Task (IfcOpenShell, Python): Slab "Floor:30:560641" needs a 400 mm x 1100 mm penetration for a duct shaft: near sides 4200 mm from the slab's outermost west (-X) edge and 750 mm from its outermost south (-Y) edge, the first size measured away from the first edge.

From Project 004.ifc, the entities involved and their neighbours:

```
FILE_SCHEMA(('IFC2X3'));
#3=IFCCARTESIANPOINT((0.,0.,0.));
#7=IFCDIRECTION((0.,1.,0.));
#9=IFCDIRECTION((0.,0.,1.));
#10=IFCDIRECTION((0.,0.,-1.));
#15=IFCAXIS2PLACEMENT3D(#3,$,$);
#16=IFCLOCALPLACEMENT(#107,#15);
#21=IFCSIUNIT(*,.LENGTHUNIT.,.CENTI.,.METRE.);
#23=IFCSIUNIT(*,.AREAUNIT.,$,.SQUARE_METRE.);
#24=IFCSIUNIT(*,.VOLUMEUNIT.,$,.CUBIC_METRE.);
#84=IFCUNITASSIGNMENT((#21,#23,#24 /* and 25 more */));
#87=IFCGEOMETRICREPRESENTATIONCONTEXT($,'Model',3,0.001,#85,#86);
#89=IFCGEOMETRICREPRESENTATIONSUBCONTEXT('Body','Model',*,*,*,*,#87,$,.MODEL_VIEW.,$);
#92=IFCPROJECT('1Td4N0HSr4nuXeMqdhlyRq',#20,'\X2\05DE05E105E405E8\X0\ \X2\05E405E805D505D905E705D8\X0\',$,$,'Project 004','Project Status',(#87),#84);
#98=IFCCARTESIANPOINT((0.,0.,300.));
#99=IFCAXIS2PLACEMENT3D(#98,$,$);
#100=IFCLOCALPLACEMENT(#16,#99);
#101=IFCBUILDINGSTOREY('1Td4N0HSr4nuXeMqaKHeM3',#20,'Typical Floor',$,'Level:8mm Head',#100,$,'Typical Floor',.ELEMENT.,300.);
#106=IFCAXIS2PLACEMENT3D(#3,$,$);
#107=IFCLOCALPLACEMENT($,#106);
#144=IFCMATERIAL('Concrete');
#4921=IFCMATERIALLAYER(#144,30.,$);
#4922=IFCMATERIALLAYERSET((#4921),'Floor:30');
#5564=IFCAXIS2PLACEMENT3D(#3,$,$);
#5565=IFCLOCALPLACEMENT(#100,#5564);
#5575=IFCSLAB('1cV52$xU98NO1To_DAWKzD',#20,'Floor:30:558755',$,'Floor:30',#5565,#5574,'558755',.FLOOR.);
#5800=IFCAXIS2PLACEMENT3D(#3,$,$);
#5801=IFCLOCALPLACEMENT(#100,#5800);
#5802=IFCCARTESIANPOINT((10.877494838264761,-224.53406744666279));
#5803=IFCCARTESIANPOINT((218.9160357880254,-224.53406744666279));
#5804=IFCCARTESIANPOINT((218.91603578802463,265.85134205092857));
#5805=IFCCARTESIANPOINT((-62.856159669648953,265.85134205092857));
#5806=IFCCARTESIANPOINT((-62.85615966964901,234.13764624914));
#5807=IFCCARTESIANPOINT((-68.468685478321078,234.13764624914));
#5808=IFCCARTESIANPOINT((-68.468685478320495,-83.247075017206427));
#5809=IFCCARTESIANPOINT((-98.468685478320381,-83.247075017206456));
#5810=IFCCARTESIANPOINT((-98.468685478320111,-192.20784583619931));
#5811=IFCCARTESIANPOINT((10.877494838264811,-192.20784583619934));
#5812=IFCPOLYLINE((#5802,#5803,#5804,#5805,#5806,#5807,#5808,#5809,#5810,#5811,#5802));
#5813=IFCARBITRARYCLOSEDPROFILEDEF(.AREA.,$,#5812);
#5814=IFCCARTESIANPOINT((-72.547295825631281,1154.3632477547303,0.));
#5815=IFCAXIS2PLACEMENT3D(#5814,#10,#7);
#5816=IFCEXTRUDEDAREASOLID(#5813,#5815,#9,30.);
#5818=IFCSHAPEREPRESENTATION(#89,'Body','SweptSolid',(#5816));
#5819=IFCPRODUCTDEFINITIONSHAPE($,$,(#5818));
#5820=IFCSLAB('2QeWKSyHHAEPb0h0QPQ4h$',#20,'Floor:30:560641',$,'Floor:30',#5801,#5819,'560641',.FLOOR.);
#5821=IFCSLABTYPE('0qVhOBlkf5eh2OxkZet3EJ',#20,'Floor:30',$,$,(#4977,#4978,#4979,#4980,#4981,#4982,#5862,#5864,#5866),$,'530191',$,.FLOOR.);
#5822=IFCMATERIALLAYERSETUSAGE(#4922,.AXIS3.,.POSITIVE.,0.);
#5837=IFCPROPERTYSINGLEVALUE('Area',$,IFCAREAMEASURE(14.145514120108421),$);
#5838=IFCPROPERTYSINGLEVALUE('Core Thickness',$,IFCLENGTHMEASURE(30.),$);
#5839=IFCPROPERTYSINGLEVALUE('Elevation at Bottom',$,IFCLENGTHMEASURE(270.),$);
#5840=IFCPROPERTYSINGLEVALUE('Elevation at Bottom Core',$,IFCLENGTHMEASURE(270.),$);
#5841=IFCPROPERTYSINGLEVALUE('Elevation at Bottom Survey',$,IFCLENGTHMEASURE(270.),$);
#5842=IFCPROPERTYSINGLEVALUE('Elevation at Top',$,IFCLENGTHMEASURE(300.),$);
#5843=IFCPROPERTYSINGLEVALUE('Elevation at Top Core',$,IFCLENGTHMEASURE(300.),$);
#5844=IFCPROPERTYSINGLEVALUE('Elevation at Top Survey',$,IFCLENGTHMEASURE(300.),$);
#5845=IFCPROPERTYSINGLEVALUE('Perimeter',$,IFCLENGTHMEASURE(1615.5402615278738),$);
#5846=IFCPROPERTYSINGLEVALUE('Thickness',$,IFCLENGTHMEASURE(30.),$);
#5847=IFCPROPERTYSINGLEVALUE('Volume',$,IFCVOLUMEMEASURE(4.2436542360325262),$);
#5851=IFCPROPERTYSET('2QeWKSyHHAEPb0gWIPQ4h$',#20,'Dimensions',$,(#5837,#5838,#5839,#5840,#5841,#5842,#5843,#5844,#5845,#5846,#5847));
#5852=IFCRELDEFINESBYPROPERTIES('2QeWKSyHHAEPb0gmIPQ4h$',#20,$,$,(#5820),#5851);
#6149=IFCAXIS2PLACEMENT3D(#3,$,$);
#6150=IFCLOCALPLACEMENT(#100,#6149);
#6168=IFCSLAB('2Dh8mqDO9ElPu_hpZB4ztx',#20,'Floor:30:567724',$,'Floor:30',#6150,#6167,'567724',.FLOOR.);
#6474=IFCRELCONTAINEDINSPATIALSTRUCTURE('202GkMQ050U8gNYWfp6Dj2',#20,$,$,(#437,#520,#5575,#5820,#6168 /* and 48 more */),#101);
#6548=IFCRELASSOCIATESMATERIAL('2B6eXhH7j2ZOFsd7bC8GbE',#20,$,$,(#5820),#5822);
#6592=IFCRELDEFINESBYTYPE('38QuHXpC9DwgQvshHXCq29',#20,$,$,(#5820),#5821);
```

```python
import numpy as np
import ifcopenshell
import ifcopenshell.api.feature
import ifcopenshell.api.geometry
import ifcopenshell.api.pset
import ifcopenshell.api.root
import ifcopenshell.geom
import ifcopenshell.util.element
import ifcopenshell.util.placement
import ifcopenshell.util.representation
import ifcopenshell.util.shape
import ifcopenshell.util.unit

model = ifcopenshell.open("Project 004.ifc")
unit_scale = ifcopenshell.util.unit.calculate_unit_scale(model)
area_scale = ifcopenshell.util.unit.calculate_unit_scale(model, "AREAUNIT")
volume_scale = ifcopenshell.util.unit.calculate_unit_scale(model, "VOLUMEUNIT")
settings = ifcopenshell.geom.settings()


def volume(element):
    """Net volume in cubic metres, openings subtracted."""
    shape = ifcopenshell.geom.create_shape(settings, element)
    return ifcopenshell.util.shape.get_volume(shape.geometry)


slab = model.by_guid("2QeWKSyHHAEPb0h0QPQ4h$")
before = volume(slab)

# Extent in the slab's own axes, in metres. The edges named are its -X and -Y sides.
slab_shape = ifcopenshell.geom.create_shape(settings, slab)
vertices = ifcopenshell.util.shape.get_vertices(slab_shape.geometry)
x_min, y_min, bottom = vertices.min(axis=0)
top = vertices[:, 2].max()

opening = ifcopenshell.api.root.create_entity(model, ifc_class="IfcOpeningElement", name="Duct shaft opening")
context = ifcopenshell.util.representation.get_context(model, "Model", "Body", "MODEL_VIEW")
width, depth = 0.4, 1.1
outline = [(0.0, 0.0), (width, 0.0), (width, depth), (0.0, depth), (0.0, 0.0)]
# Overshoot both faces by 50 mm so the cut is clean.
shape = ifcopenshell.api.geometry.add_slab_representation(
    model, context=context, depth=top - bottom + 0.1, polyline=outline
)
ifcopenshell.api.geometry.assign_representation(model, product=opening, representation=shape)

matrix = ifcopenshell.util.placement.get_local_placement(slab.ObjectPlacement)
matrix[:, 3] = matrix @ np.append(np.array([x_min + 4.2, y_min + 0.75, bottom - 0.05]) / unit_scale, 1.0)
ifcopenshell.api.geometry.edit_object_placement(model, product=opening, matrix=matrix, is_si=False)
ifcopenshell.api.feature.add_feature(model, feature=opening, element=slab)

after = volume(slab)

# Update the slab's stored quantities.
pset = model.by_id(ifcopenshell.util.element.get_pset(slab, "Dimensions", should_inherit=False)["id"])
ifcopenshell.api.pset.edit_pset(model, pset=pset, properties={
    "Area": model.create_entity("IfcAreaMeasure", after / (top - bottom) / area_scale),
    "Volume": model.create_entity("IfcVolumeMeasure", after / volume_scale),
})

print(f"slab volume {before:.3f} -> {after:.3f} m3")

model.write("Project 004-out.ifc")
```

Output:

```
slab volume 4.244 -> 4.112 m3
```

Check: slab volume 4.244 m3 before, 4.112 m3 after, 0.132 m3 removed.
